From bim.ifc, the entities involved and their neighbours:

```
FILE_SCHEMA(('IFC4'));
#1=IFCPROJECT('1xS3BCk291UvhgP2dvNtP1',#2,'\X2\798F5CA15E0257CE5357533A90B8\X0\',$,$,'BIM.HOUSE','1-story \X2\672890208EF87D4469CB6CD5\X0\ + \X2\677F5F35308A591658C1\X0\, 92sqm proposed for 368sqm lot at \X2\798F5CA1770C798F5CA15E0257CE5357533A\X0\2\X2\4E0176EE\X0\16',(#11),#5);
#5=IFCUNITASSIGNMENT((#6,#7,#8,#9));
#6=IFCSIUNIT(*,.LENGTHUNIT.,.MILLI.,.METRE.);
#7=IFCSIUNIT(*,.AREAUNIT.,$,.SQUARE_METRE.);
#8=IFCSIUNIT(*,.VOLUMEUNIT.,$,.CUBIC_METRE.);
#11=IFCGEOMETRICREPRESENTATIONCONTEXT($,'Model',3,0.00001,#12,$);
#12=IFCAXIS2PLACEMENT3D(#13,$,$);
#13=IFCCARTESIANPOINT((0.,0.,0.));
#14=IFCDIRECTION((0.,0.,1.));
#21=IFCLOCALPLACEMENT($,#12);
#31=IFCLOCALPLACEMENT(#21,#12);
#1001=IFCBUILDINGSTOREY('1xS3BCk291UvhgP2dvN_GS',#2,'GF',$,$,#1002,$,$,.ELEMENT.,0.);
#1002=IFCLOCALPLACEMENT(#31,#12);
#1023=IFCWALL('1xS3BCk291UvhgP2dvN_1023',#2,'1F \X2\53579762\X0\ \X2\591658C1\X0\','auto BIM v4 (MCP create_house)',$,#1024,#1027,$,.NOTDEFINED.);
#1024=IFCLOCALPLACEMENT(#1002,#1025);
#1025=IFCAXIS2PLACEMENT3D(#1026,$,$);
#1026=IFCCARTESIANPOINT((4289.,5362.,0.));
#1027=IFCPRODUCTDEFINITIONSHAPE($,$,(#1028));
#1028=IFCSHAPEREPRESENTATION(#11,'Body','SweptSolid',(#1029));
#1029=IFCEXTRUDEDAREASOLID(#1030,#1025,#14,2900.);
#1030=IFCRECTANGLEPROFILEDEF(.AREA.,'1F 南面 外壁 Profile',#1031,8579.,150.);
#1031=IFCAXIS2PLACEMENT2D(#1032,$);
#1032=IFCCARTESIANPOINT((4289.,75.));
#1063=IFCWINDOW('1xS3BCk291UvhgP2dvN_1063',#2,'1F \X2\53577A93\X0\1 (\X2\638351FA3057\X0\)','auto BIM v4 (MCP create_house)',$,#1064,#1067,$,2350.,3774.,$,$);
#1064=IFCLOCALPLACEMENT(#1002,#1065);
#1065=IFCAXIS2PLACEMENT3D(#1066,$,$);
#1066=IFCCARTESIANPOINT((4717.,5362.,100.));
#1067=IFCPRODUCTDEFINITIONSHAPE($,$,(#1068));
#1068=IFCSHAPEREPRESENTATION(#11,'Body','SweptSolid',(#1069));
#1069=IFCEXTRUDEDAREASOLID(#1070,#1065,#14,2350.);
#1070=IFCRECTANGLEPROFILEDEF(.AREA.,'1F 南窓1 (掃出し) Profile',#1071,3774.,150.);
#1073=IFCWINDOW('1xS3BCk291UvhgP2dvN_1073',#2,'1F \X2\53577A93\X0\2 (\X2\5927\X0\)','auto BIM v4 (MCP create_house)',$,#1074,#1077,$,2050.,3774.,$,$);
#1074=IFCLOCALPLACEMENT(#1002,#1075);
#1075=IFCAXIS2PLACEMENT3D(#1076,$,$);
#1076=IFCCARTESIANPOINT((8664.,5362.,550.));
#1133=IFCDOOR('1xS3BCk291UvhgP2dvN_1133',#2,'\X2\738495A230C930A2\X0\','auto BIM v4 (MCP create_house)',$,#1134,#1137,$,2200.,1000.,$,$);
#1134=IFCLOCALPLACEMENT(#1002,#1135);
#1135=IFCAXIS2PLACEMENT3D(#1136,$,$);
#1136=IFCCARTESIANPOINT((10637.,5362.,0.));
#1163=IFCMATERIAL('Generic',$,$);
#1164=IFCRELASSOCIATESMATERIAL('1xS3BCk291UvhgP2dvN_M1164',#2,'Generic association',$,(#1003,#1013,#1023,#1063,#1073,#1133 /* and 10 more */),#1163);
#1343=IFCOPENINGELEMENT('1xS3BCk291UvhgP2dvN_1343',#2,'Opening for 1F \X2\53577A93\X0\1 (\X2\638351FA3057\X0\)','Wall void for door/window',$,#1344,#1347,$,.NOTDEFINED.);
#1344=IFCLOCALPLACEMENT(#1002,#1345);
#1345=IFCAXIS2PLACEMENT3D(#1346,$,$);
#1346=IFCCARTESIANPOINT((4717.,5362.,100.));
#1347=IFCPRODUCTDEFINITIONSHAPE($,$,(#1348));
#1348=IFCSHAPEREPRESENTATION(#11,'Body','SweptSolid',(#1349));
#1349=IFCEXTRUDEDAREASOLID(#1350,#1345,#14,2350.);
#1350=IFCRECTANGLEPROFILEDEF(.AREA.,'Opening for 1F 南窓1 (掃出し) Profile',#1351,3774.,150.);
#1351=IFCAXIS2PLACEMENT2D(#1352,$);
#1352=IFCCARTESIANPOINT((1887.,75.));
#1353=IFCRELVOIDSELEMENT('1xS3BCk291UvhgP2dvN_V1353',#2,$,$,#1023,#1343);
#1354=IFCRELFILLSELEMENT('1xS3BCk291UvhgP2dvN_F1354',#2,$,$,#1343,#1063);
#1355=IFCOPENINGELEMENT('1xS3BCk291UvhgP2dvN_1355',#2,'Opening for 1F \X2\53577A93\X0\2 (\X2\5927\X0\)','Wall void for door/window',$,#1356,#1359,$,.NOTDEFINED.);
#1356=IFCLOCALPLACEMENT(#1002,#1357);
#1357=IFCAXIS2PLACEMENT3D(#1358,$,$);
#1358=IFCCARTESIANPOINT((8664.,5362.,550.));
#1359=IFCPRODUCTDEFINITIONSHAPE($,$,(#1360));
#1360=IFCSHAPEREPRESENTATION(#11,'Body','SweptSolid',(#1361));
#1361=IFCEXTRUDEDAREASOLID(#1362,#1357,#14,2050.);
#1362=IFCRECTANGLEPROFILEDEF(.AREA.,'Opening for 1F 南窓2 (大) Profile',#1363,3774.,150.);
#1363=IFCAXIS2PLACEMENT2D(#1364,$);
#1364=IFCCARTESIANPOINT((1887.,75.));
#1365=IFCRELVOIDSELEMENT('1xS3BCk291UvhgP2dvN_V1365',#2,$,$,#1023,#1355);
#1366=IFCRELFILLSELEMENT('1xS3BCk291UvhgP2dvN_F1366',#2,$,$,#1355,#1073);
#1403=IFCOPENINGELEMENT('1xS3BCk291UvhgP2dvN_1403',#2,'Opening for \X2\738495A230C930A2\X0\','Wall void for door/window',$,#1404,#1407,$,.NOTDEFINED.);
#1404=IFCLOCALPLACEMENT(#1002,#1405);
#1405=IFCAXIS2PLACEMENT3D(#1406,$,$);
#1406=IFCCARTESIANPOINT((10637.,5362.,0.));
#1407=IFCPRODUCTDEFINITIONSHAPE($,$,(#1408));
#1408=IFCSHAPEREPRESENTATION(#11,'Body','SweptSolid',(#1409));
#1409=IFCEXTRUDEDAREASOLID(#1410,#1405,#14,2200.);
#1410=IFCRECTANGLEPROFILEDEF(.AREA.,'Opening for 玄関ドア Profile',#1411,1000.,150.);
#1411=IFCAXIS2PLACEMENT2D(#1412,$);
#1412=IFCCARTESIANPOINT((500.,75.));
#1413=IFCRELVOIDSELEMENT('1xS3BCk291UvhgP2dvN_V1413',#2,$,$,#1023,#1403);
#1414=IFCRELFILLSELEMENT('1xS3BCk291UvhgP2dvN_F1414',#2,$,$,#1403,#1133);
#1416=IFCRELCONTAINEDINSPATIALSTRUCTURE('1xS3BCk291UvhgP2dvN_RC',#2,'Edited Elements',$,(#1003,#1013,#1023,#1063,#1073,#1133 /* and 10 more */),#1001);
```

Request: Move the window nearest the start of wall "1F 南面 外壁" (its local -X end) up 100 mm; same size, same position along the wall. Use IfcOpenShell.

```python
import numpy as np
import ifcopenshell
import ifcopenshell.api.geometry
import ifcopenshell.util.placement
import ifcopenshell.util.unit

model = ifcopenshell.open("bim.ifc")
unit_scale = ifcopenshell.util.unit.calculate_unit_scale(model)

window = model.by_id(1063)
opening = window.FillsVoids[0].RelatingOpeningElement
dz = 0.1 / unit_scale

shift = np.array([0.0, 0.0, dz])
# The window is not placed relative to its opening, so move both.
for product in (opening, window):
    matrix = ifcopenshell.util.placement.get_local_placement(product.ObjectPlacement)
    matrix[:3, 3] += shift
    ifcopenshell.api.geometry.edit_object_placement(model, product=product, matrix=matrix, is_si=False)

print(f"moved by {dz * unit_scale:+.3f} m")

model.write("bim_rev.ifc")
```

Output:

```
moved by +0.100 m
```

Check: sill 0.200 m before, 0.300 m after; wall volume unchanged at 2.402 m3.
